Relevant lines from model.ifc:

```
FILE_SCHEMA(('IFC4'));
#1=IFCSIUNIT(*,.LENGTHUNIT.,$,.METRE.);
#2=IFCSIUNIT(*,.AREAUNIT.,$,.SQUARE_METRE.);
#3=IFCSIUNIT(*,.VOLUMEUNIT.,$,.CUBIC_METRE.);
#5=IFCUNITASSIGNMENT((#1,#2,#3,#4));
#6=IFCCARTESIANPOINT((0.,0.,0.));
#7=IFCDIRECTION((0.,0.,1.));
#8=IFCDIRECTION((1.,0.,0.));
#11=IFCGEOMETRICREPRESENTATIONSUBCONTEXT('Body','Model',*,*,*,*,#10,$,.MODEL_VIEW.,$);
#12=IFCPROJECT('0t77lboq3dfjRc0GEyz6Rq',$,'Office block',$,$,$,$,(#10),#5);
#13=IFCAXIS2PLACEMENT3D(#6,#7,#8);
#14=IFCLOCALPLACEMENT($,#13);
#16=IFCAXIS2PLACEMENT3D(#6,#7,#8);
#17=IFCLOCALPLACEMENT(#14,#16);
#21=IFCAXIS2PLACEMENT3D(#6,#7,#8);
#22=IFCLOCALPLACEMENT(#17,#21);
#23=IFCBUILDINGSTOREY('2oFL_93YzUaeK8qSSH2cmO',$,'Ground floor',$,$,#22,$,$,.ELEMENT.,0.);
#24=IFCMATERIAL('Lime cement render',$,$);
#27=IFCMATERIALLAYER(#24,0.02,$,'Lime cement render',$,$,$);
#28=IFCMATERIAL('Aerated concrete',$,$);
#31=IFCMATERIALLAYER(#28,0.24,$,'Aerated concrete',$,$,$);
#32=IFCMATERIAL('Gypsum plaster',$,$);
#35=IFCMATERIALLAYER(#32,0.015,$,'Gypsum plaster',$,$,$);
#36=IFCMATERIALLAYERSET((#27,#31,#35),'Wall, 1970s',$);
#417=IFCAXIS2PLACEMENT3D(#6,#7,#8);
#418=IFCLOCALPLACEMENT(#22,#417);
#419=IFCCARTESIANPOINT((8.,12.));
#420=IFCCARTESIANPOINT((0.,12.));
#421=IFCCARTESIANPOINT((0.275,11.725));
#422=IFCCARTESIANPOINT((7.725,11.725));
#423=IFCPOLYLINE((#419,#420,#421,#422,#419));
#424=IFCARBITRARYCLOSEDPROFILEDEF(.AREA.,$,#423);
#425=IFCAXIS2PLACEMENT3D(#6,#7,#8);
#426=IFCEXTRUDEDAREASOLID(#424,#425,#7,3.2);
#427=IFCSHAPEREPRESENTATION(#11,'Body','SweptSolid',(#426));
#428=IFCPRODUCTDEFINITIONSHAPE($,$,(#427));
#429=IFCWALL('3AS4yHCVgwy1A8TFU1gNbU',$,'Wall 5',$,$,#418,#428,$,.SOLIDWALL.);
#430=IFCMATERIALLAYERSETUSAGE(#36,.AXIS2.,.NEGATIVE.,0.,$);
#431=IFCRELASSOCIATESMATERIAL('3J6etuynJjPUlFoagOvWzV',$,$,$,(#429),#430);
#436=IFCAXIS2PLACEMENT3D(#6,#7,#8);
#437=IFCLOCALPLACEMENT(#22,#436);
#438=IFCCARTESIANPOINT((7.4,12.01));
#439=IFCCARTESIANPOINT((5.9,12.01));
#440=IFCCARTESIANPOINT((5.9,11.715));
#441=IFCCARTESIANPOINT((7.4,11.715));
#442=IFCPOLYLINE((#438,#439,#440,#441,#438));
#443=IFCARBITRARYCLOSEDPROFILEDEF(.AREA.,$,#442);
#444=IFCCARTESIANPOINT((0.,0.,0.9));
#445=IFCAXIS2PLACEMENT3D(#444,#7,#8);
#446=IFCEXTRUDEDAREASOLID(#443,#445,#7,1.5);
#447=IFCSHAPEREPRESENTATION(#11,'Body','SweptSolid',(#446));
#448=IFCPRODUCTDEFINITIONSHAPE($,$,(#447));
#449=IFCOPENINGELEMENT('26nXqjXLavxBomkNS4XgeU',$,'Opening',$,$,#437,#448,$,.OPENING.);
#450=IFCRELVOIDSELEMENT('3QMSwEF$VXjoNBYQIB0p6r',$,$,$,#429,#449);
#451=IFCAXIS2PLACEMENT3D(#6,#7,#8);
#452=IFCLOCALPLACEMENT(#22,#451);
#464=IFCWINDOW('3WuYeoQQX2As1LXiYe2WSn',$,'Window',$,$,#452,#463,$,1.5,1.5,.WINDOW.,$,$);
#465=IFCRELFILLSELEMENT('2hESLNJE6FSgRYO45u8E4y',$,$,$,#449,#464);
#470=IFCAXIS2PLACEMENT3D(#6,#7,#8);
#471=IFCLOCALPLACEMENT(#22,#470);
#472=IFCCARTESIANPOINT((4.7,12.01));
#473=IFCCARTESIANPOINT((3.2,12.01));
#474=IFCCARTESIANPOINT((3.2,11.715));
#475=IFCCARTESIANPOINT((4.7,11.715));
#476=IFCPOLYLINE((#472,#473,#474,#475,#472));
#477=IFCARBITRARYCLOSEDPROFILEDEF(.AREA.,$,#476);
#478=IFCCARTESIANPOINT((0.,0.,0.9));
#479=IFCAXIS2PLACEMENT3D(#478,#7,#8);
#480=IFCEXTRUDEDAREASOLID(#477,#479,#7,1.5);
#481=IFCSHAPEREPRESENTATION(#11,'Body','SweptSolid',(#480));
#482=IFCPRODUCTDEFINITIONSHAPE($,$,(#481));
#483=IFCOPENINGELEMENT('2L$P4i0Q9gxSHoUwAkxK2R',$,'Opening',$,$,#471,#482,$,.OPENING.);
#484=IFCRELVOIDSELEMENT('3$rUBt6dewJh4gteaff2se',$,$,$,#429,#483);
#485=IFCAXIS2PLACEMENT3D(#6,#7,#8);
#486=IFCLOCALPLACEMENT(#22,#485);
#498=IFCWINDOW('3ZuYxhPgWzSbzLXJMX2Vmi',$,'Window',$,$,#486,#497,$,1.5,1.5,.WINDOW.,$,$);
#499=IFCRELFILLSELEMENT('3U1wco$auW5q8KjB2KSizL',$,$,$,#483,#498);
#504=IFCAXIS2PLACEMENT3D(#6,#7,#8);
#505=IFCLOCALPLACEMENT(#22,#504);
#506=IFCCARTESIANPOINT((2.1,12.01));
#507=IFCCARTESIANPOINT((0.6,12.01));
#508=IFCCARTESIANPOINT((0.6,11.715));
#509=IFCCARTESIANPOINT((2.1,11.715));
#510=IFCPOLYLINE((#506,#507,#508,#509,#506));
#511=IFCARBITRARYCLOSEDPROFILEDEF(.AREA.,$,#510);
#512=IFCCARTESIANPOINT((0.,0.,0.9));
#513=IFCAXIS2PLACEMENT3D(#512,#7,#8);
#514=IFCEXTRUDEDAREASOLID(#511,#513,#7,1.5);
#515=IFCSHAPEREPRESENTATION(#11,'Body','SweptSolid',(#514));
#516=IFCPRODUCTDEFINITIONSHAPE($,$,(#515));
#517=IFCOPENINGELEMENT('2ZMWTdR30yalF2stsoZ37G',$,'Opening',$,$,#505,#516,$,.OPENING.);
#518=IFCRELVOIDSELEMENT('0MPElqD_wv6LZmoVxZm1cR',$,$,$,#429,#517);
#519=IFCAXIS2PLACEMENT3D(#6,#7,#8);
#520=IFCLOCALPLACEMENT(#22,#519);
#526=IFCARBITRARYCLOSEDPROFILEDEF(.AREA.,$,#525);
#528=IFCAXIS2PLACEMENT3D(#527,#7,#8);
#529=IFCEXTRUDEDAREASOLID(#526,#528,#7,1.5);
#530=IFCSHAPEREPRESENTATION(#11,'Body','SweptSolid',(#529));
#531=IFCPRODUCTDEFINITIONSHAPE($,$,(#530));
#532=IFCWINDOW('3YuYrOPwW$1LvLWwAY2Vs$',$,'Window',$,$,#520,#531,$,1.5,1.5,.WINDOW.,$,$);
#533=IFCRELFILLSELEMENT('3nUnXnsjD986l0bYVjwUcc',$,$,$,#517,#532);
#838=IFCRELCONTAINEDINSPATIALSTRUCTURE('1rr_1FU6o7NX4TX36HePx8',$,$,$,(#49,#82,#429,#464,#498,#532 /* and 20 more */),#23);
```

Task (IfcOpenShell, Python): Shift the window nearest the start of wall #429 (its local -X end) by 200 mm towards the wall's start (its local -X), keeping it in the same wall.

```python
import ifcopenshell
import ifcopenshell.api.geometry
import ifcopenshell.util.placement
import ifcopenshell.util.unit

model = ifcopenshell.open("model.ifc")
unit_scale = ifcopenshell.util.unit.calculate_unit_scale(model)

window = model.by_id(532)
opening = window.FillsVoids[0].RelatingOpeningElement
wall = opening.VoidsElements[0].RelatingBuildingElement

wall_matrix = ifcopenshell.util.placement.get_local_placement(wall.ObjectPlacement)
shift = wall_matrix[:3, 0] * -0.2 / unit_scale
before = ifcopenshell.util.placement.get_local_placement(window.ObjectPlacement)[:3, 3].copy()

# The window is not placed relative to its opening, so move both.
for product in (opening, window):
    matrix = ifcopenshell.util.placement.get_local_placement(product.ObjectPlacement)
    matrix[:3, 3] += shift
    ifcopenshell.api.geometry.edit_object_placement(model, product=product, matrix=matrix, is_si=False)

after = ifcopenshell.util.placement.get_local_placement(window.ObjectPlacement)[:3, 3]
print("window moved by", (after - before).round(3) + 0.0)

model.write("model_v2.ifc")
```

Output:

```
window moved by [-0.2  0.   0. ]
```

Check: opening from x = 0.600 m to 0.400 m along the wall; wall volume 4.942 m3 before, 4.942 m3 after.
